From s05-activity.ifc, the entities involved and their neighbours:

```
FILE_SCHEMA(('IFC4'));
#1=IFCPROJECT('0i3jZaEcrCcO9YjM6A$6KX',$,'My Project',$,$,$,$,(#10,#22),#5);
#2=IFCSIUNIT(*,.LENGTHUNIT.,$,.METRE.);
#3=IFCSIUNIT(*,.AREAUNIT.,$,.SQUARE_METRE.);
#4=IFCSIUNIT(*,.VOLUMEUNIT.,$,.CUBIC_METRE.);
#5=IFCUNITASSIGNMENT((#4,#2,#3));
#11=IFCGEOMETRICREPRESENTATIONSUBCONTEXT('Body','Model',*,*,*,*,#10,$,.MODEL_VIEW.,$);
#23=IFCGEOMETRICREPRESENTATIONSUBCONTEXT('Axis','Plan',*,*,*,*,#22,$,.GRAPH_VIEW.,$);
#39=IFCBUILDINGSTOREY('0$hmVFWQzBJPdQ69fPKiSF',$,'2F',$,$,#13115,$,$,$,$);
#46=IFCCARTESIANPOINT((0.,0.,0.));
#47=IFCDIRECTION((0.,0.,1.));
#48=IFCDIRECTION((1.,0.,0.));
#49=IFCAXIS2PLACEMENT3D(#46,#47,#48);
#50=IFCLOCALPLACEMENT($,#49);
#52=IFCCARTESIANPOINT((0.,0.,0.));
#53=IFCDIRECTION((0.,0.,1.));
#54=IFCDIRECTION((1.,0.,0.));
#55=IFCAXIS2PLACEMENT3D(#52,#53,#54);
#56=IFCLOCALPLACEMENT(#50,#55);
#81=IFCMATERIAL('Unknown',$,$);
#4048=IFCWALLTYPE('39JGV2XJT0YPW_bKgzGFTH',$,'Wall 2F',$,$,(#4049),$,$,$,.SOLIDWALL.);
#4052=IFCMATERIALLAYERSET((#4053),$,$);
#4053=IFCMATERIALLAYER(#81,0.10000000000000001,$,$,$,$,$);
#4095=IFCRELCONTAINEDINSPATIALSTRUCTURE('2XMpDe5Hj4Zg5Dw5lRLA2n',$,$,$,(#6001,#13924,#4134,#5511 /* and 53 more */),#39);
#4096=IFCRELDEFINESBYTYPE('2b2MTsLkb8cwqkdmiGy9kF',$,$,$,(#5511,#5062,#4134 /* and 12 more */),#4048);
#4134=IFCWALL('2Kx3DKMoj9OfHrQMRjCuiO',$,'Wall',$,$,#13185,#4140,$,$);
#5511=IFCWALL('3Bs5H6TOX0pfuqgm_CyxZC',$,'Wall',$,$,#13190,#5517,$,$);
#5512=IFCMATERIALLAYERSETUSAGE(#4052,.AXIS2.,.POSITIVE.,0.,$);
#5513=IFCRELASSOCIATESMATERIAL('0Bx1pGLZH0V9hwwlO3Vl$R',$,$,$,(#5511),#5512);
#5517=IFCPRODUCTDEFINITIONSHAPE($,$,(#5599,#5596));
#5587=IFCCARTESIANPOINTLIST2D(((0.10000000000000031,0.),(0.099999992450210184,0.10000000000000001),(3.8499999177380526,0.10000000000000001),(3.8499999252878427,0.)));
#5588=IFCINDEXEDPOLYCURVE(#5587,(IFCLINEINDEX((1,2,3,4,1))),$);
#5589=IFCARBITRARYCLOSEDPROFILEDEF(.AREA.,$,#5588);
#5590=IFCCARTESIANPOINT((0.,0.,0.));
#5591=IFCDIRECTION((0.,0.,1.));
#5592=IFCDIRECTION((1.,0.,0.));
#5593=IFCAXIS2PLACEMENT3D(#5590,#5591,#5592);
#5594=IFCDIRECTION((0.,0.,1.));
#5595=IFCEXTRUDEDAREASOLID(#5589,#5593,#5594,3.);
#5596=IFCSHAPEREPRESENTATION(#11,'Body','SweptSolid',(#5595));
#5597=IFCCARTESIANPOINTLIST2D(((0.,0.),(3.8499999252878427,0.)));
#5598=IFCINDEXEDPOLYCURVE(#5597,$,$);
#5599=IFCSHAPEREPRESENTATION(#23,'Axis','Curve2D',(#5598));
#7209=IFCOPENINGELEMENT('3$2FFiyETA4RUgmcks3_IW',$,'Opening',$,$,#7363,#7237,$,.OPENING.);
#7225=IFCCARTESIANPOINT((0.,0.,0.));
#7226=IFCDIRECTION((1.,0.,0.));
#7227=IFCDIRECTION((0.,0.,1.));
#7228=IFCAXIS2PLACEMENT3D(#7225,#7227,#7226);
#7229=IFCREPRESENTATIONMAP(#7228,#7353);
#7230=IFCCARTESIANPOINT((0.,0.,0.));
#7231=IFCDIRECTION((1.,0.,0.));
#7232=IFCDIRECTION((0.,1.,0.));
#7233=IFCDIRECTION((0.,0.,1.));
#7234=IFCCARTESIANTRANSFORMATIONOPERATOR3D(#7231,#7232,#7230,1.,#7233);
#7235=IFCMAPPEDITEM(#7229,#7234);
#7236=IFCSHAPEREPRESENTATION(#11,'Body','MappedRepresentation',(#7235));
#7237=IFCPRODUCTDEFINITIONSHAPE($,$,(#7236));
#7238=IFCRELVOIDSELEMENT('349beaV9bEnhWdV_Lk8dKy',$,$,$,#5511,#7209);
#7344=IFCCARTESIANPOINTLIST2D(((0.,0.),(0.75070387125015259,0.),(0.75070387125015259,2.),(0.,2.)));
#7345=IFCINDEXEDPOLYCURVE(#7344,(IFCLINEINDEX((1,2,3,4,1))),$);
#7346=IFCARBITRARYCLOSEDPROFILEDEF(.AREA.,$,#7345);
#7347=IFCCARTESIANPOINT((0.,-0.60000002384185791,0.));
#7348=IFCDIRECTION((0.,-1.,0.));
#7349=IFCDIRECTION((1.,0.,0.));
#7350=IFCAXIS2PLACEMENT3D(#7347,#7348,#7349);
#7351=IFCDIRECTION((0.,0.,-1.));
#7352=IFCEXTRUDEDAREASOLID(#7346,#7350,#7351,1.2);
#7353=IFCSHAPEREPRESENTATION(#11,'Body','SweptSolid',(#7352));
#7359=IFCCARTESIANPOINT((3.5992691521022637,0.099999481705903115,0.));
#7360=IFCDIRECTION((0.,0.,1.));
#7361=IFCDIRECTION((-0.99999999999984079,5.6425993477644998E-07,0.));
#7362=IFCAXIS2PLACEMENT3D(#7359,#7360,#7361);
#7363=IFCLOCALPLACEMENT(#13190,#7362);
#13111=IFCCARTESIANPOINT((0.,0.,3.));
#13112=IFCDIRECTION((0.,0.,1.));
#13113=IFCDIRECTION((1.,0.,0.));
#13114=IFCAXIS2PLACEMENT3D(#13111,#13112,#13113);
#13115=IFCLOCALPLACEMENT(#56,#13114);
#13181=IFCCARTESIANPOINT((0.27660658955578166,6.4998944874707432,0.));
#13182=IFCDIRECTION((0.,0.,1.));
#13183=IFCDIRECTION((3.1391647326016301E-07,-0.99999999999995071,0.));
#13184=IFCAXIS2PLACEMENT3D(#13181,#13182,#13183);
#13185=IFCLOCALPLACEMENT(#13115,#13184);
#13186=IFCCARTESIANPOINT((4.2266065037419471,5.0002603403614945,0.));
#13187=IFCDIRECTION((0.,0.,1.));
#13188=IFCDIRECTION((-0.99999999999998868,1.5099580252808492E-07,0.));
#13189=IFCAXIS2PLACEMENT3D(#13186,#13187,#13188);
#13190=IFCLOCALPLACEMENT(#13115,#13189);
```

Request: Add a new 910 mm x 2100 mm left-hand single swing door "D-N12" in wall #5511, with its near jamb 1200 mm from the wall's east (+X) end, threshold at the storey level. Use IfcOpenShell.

```python
import numpy as np
import ifcopenshell
import ifcopenshell.api.feature
import ifcopenshell.api.geometry
import ifcopenshell.api.root
import ifcopenshell.api.spatial
import ifcopenshell.geom
import ifcopenshell.util.element
import ifcopenshell.util.placement
import ifcopenshell.util.representation
import ifcopenshell.util.shape
import ifcopenshell.util.unit

model = ifcopenshell.open("s05-activity.ifc")
unit_scale = ifcopenshell.util.unit.calculate_unit_scale(model)
settings = ifcopenshell.geom.settings()


def volume(element):
    """Net volume in cubic metres, openings subtracted."""
    shape = ifcopenshell.geom.create_shape(settings, element)
    return ifcopenshell.util.shape.get_volume(shape.geometry)


wall = model.by_guid("3Bs5H6TOX0pfuqgm_CyxZC")
storey = ifcopenshell.util.element.get_container(wall, ifc_class="IfcBuildingStorey")
context = ifcopenshell.util.representation.get_context(model, "Model", "Body", "MODEL_VIEW")
before = volume(wall)

width, height, from_end, sill = 0.91, 2.1, 1.2, 0.0  # metres

# The wall runs along its own X axis, and the end named is its -X end.
wall_shape = ifcopenshell.geom.create_shape(settings, wall)
x, y, z = ifcopenshell.util.shape.get_vertices(wall_shape.geometry).T
start = x.min() + from_end
face, thickness = float(y.min()), float(y.max() - y.min())
wall_matrix = ifcopenshell.util.placement.get_local_placement(wall.ObjectPlacement)
level = ifcopenshell.util.placement.get_local_placement(storey.ObjectPlacement)[2, 3]


def in_wall(x, y):
    """Placement at x, y metres in the wall's axes, at sill height."""
    matrix = wall_matrix.copy()
    matrix[:, 3] = wall_matrix @ np.array([x / unit_scale, y / unit_scale, 0.0, 1.0])
    matrix[2, 3] = level + sill / unit_scale
    return matrix


# Opening: a box that overshoots both wall faces by 50 mm.
opening = ifcopenshell.api.root.create_entity(model, ifc_class="IfcOpeningElement", predefined_type="OPENING")
box = ifcopenshell.api.geometry.add_wall_representation(
    model, context=context, length=width, height=height, thickness=thickness + 0.1
)
ifcopenshell.api.geometry.assign_representation(model, product=opening, representation=box)
ifcopenshell.api.geometry.edit_object_placement(model, product=opening, matrix=in_wall(start, face - 0.05), is_si=False)
ifcopenshell.api.feature.add_feature(model, feature=opening, element=wall)

door = ifcopenshell.api.root.create_entity(model, ifc_class="IfcDoor", name="D-N12", predefined_type="DOOR")
door.OverallWidth, door.OverallHeight = width / unit_scale, height / unit_scale
door.OperationType = "SINGLE_SWING_LEFT"
body = ifcopenshell.api.geometry.add_door_representation(
    model,
    context=context,
    overall_width=door.OverallWidth,
    overall_height=door.OverallHeight,
    operation_type="SINGLE_SWING_LEFT",
    lining_properties={"LiningDepth": thickness / unit_scale, "ThresholdDepth": thickness / unit_scale},
)
ifcopenshell.api.geometry.assign_representation(model, product=door, representation=body)
ifcopenshell.api.spatial.assign_container(model, products=[door], relating_structure=storey)
ifcopenshell.api.feature.add_filling(model, opening=opening, element=door)

# The lining spans the wall, so the door starts at the wall face.
ifcopenshell.api.geometry.edit_object_placement(model, product=door, matrix=in_wall(start, face), is_si=False)

after = volume(wall)

print(f"wall volume {before:.3f} -> {after:.3f} m3")

model.write("s05-activity_updated.ifc")
```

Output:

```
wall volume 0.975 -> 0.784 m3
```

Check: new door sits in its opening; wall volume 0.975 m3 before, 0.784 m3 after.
